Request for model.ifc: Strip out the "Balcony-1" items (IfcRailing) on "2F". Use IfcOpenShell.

First a look at what the model holds.

```python
import ifcopenshell
import ifcopenshell.util.element

model = ifcopenshell.open("model.ifc")
print(model.schema)
storey = next(s for s in model.by_type("IfcBuildingStorey") if s.Name == "2F")
railings = [e for e in ifcopenshell.util.element.get_decomposition(storey) if e.is_a("IfcRailing")]
seen = {}
for e in railings:
    element_type = ifcopenshell.util.element.get_type(e)
    name = element_type.Name if element_type not in (None, e) else None
    seen[name] = seen.get(name, 0) + 1
for name, count in sorted(seen.items(), key=str):
    print(count, "x", name)
```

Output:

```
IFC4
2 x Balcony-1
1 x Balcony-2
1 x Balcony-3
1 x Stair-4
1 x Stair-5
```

```python
import ifcopenshell
import ifcopenshell.api.root
import ifcopenshell.util.element

model = ifcopenshell.open("model.ifc")

storey = next(s for s in model.by_type("IfcBuildingStorey") if s.Name == "2F")
railings = [e for e in ifcopenshell.util.element.get_decomposition(storey) if e.is_a("IfcRailing")]
targets = [e for e in railings if (t := ifcopenshell.util.element.get_type(e)) not in (None, e) and t.Name == "Balcony-1"]

for e in targets:
    ifcopenshell.api.root.remove_product(model, product=e)
print(len(targets), "removed")

model.write("model_updated.ifc")
```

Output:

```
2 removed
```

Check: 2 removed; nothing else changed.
